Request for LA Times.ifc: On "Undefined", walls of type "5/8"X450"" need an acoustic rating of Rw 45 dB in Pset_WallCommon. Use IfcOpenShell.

First a look at what the model holds.

```python
import ifcopenshell
import ifcopenshell.util.element

model = ifcopenshell.open("LA Times.ifc")
print(model.schema)
storey = next(s for s in model.by_type("IfcBuildingStorey") if s.Name == "Undefined")
walls = [e for e in ifcopenshell.util.element.get_decomposition(storey) if e.is_a("IfcWall")]
seen = {}
for e in walls:
    element_type = ifcopenshell.util.element.get_type(e)
    key = (element_type.Name if element_type != e and element_type else None, ifcopenshell.util.element.get_pset(e, "Pset_WallCommon", "AcousticRating"))
    seen[key] = seen.get(key, 0) + 1
for (name, value), count in sorted(seen.items(), key=str):
    print(count, "x", name, "|", value)
```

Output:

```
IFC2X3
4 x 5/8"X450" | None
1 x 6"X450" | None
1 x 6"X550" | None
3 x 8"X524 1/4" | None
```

```python
import ifcopenshell
import ifcopenshell.api.pset
import ifcopenshell.util.element

model = ifcopenshell.open("LA Times.ifc")

storey = next(s for s in model.by_type("IfcBuildingStorey") if s.Name == "Undefined")
walls = [e for e in ifcopenshell.util.element.get_decomposition(storey) if e.is_a("IfcWall")]

count = 0
for e in walls:
    element_type = ifcopenshell.util.element.get_type(e)
    if element_type in (None, e) or element_type.Name != '5/8"X450"':
        continue
    found = ifcopenshell.util.element.get_pset(e, "Pset_WallCommon", should_inherit=False)
    if found:
        pset = model.by_id(found["id"])
        if len(ifcopenshell.util.element.get_elements_by_pset(pset)) > 1:
            pset = ifcopenshell.api.pset.unshare_pset(model, products=[e], pset=pset)[0]
    else:
        pset = ifcopenshell.api.pset.add_pset(model, product=e, name="Pset_WallCommon")
    ifcopenshell.api.pset.edit_pset(model, pset=pset, properties={"AcousticRating": "Rw 45 dB"})
    count += 1

print(count, "walls updated")

model.write("LA Times_v2.ifc")
```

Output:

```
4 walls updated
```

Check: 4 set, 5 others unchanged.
